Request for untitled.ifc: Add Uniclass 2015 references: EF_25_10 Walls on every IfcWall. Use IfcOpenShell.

First a look at what the model holds.

```python
import ifcopenshell

model = ifcopenshell.open("untitled.ifc")
print(model.schema)
print("classifications:", [c.Name for c in model.by_type("IfcClassification")])
for ifc_class in ("IfcDoor", "IfcRoof", "IfcStair", "IfcWall", "IfcWindow"):
    print(ifc_class, len(model.by_type(ifc_class)))
```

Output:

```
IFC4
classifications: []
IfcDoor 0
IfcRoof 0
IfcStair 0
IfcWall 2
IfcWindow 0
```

```python
import ifcopenshell
import ifcopenshell.api.classification

model = ifcopenshell.open("untitled.ifc")

system = ifcopenshell.api.classification.add_classification(model, classification="Uniclass 2015")

codes = {
    "IfcWall": ("EF_25_10", "Walls"),
}
for ifc_class, (code, name) in codes.items():
    products = model.by_type(ifc_class)
    ifcopenshell.api.classification.add_reference(
        model, products=products, classification=system, identification=code, name=name
    )
    print(code, len(products))

model.write("untitled_edited.ifc")
```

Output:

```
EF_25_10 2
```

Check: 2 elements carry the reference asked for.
